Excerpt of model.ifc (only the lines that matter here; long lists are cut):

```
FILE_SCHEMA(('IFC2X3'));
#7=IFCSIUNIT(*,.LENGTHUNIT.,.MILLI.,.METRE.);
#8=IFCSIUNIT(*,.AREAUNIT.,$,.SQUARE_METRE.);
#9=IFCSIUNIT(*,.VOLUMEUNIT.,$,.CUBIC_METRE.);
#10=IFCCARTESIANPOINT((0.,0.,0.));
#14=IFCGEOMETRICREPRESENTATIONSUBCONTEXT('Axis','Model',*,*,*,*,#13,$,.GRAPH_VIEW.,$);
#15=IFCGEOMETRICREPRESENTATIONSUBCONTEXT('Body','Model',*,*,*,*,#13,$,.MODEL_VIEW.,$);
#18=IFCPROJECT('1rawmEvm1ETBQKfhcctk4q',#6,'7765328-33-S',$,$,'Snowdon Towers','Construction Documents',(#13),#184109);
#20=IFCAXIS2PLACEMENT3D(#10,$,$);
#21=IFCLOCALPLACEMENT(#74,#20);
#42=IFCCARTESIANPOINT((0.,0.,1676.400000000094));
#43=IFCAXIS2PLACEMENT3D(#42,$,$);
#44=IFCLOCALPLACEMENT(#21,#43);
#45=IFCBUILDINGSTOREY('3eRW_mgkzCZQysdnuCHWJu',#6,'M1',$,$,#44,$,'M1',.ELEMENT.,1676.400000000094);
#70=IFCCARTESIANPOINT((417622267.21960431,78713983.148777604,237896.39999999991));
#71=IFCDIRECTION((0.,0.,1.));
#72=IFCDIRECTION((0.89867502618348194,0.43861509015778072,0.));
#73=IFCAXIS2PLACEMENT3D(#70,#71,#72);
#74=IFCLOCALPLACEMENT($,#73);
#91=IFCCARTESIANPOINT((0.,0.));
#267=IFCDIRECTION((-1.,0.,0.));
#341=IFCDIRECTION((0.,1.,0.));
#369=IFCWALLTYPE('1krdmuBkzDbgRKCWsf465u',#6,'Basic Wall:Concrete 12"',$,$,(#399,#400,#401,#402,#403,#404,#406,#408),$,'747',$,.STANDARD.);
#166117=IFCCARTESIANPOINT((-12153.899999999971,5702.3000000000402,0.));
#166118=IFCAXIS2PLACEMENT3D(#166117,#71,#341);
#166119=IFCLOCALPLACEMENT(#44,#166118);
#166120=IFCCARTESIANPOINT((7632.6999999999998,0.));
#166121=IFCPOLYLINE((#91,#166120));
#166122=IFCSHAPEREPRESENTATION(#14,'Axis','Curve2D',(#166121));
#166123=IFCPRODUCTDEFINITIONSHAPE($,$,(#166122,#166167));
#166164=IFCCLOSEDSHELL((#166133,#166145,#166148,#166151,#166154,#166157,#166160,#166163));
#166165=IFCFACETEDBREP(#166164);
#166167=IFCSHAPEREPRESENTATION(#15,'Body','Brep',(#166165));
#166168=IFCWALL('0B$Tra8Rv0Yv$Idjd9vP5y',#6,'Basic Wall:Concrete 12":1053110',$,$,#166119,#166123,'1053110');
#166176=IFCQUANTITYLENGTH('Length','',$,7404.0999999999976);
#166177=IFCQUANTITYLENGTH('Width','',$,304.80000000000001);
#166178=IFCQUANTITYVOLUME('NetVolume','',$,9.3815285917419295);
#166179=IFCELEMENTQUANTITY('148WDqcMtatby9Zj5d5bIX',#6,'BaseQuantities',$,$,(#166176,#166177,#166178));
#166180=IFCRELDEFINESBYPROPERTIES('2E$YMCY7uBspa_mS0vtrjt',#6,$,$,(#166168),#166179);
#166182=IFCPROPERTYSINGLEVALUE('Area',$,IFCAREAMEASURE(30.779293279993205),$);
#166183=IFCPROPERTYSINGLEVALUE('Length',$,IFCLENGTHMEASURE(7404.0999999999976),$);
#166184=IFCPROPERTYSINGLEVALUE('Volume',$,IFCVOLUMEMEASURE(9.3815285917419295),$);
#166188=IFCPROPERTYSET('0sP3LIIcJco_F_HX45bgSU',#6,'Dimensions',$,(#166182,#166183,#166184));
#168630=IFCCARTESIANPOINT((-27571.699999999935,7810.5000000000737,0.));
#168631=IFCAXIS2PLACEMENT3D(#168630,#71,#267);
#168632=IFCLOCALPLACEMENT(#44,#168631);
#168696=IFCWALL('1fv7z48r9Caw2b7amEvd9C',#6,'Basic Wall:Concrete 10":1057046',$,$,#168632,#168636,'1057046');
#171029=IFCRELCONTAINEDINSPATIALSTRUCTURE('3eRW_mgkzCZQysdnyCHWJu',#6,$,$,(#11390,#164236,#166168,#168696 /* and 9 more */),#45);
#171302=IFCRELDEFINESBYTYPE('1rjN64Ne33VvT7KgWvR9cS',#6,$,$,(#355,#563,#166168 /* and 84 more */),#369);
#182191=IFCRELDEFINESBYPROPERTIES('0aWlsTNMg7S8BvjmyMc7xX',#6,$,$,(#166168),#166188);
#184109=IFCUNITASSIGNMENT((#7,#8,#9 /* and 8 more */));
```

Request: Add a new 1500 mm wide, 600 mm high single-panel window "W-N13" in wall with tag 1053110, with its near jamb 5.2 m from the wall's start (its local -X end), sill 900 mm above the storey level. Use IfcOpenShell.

```python
import numpy as np
import ifcopenshell
import ifcopenshell.api.feature
import ifcopenshell.api.geometry
import ifcopenshell.api.pset
import ifcopenshell.api.root
import ifcopenshell.api.spatial
import ifcopenshell.api.type
import ifcopenshell.geom
import ifcopenshell.util.element
import ifcopenshell.util.placement
import ifcopenshell.util.representation
import ifcopenshell.util.shape
import ifcopenshell.util.unit

model = ifcopenshell.open("model.ifc")
unit_scale = ifcopenshell.util.unit.calculate_unit_scale(model)
area_scale = ifcopenshell.util.unit.calculate_unit_scale(model, "AREAUNIT")
volume_scale = ifcopenshell.util.unit.calculate_unit_scale(model, "VOLUMEUNIT")
settings = ifcopenshell.geom.settings()


def volume(element):
    """Net volume in cubic metres, openings subtracted."""
    shape = ifcopenshell.geom.create_shape(settings, element)
    return ifcopenshell.util.shape.get_volume(shape.geometry)


wall = model.by_guid("0B$Tra8Rv0Yv$Idjd9vP5y")
storey = ifcopenshell.util.element.get_container(wall, ifc_class="IfcBuildingStorey")
context = ifcopenshell.util.representation.get_context(model, "Model", "Body", "MODEL_VIEW")
before = volume(wall)

width, height, from_end, sill = 1.5, 0.6, 5.2, 0.9  # metres

# The wall runs along its own X axis, and the end named is its -X end.
wall_shape = ifcopenshell.geom.create_shape(settings, wall)
x, y, z = ifcopenshell.util.shape.get_vertices(wall_shape.geometry).T
start = x.min() + from_end
face, thickness = float(y.min()), float(y.max() - y.min())
wall_matrix = ifcopenshell.util.placement.get_local_placement(wall.ObjectPlacement)
level = ifcopenshell.util.placement.get_local_placement(storey.ObjectPlacement)[2, 3]


def in_wall(x, y):
    """Placement at x, y metres in the wall's axes, at sill height."""
    matrix = wall_matrix.copy()
    matrix[:, 3] = wall_matrix @ np.array([x / unit_scale, y / unit_scale, 0.0, 1.0])
    matrix[2, 3] = level + sill / unit_scale
    return matrix


# Opening: a box that overshoots both wall faces by 50 mm.
opening = ifcopenshell.api.root.create_entity(model, ifc_class="IfcOpeningElement")
box = ifcopenshell.api.geometry.add_wall_representation(
    model, context=context, length=width, height=height, thickness=thickness + 0.1
)
ifcopenshell.api.geometry.assign_representation(model, product=opening, representation=box)
ifcopenshell.api.geometry.edit_object_placement(model, product=opening, matrix=in_wall(start, face - 0.05), is_si=False)
ifcopenshell.api.feature.add_feature(model, feature=opening, element=wall)

window = ifcopenshell.api.root.create_entity(model, ifc_class="IfcWindow", name="W-N13")
window.OverallWidth, window.OverallHeight = width / unit_scale, height / unit_scale
body = ifcopenshell.api.geometry.add_window_representation(
    model,
    context=context,
    overall_width=window.OverallWidth,
    overall_height=window.OverallHeight,
    partition_type="SINGLE_PANEL",
)
ifcopenshell.api.geometry.assign_representation(model, product=window, representation=body)
ifcopenshell.api.spatial.assign_container(model, products=[window], relating_structure=storey)
fills = ifcopenshell.api.feature.add_filling(model, opening=opening, element=window)
fills.OwnerHistory = window.OwnerHistory  # required in IFC2X3

# IFC2X3 keeps the operation on the window style.
style = ifcopenshell.api.root.create_entity(model, ifc_class="IfcWindowStyle", name="W-N13")
style.OperationType, style.ConstructionType = "SINGLE_PANEL", "NOTDEFINED"
style.ParameterTakesPrecedence = style.Sizeable = False
ifcopenshell.api.type.assign_type(model, related_objects=[window], relating_type=style)

# Centre the window in the wall's thickness.
ifcopenshell.api.geometry.edit_object_placement(model, product=window, matrix=in_wall(start, face), is_si=False)
window_shape = ifcopenshell.geom.create_shape(settings, window)
depth = ifcopenshell.util.shape.get_vertices(window_shape.geometry)[:, 1]
offset = face + thickness / 2 - (depth.min() + depth.max()) / 2
ifcopenshell.api.geometry.edit_object_placement(model, product=window, matrix=in_wall(start, offset), is_si=False)

after = volume(wall)

# Update the wall's stored quantities.
qto = model.by_id(ifcopenshell.util.element.get_pset(wall, "BaseQuantities", should_inherit=False)["id"])
ifcopenshell.api.pset.edit_qto(model, qto=qto, properties={"NetVolume": after / volume_scale})
pset = model.by_id(ifcopenshell.util.element.get_pset(wall, "Dimensions", should_inherit=False)["id"])
ifcopenshell.api.pset.edit_pset(model, pset=pset, properties={
    "Area": model.create_entity("IfcAreaMeasure", after / thickness / area_scale),
    "Volume": model.create_entity("IfcVolumeMeasure", after / volume_scale),
})

print(f"wall volume {before:.3f} -> {after:.3f} m3")

model.write("model_v2.ifc")
```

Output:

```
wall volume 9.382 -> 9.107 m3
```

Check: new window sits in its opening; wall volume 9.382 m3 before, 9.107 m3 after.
